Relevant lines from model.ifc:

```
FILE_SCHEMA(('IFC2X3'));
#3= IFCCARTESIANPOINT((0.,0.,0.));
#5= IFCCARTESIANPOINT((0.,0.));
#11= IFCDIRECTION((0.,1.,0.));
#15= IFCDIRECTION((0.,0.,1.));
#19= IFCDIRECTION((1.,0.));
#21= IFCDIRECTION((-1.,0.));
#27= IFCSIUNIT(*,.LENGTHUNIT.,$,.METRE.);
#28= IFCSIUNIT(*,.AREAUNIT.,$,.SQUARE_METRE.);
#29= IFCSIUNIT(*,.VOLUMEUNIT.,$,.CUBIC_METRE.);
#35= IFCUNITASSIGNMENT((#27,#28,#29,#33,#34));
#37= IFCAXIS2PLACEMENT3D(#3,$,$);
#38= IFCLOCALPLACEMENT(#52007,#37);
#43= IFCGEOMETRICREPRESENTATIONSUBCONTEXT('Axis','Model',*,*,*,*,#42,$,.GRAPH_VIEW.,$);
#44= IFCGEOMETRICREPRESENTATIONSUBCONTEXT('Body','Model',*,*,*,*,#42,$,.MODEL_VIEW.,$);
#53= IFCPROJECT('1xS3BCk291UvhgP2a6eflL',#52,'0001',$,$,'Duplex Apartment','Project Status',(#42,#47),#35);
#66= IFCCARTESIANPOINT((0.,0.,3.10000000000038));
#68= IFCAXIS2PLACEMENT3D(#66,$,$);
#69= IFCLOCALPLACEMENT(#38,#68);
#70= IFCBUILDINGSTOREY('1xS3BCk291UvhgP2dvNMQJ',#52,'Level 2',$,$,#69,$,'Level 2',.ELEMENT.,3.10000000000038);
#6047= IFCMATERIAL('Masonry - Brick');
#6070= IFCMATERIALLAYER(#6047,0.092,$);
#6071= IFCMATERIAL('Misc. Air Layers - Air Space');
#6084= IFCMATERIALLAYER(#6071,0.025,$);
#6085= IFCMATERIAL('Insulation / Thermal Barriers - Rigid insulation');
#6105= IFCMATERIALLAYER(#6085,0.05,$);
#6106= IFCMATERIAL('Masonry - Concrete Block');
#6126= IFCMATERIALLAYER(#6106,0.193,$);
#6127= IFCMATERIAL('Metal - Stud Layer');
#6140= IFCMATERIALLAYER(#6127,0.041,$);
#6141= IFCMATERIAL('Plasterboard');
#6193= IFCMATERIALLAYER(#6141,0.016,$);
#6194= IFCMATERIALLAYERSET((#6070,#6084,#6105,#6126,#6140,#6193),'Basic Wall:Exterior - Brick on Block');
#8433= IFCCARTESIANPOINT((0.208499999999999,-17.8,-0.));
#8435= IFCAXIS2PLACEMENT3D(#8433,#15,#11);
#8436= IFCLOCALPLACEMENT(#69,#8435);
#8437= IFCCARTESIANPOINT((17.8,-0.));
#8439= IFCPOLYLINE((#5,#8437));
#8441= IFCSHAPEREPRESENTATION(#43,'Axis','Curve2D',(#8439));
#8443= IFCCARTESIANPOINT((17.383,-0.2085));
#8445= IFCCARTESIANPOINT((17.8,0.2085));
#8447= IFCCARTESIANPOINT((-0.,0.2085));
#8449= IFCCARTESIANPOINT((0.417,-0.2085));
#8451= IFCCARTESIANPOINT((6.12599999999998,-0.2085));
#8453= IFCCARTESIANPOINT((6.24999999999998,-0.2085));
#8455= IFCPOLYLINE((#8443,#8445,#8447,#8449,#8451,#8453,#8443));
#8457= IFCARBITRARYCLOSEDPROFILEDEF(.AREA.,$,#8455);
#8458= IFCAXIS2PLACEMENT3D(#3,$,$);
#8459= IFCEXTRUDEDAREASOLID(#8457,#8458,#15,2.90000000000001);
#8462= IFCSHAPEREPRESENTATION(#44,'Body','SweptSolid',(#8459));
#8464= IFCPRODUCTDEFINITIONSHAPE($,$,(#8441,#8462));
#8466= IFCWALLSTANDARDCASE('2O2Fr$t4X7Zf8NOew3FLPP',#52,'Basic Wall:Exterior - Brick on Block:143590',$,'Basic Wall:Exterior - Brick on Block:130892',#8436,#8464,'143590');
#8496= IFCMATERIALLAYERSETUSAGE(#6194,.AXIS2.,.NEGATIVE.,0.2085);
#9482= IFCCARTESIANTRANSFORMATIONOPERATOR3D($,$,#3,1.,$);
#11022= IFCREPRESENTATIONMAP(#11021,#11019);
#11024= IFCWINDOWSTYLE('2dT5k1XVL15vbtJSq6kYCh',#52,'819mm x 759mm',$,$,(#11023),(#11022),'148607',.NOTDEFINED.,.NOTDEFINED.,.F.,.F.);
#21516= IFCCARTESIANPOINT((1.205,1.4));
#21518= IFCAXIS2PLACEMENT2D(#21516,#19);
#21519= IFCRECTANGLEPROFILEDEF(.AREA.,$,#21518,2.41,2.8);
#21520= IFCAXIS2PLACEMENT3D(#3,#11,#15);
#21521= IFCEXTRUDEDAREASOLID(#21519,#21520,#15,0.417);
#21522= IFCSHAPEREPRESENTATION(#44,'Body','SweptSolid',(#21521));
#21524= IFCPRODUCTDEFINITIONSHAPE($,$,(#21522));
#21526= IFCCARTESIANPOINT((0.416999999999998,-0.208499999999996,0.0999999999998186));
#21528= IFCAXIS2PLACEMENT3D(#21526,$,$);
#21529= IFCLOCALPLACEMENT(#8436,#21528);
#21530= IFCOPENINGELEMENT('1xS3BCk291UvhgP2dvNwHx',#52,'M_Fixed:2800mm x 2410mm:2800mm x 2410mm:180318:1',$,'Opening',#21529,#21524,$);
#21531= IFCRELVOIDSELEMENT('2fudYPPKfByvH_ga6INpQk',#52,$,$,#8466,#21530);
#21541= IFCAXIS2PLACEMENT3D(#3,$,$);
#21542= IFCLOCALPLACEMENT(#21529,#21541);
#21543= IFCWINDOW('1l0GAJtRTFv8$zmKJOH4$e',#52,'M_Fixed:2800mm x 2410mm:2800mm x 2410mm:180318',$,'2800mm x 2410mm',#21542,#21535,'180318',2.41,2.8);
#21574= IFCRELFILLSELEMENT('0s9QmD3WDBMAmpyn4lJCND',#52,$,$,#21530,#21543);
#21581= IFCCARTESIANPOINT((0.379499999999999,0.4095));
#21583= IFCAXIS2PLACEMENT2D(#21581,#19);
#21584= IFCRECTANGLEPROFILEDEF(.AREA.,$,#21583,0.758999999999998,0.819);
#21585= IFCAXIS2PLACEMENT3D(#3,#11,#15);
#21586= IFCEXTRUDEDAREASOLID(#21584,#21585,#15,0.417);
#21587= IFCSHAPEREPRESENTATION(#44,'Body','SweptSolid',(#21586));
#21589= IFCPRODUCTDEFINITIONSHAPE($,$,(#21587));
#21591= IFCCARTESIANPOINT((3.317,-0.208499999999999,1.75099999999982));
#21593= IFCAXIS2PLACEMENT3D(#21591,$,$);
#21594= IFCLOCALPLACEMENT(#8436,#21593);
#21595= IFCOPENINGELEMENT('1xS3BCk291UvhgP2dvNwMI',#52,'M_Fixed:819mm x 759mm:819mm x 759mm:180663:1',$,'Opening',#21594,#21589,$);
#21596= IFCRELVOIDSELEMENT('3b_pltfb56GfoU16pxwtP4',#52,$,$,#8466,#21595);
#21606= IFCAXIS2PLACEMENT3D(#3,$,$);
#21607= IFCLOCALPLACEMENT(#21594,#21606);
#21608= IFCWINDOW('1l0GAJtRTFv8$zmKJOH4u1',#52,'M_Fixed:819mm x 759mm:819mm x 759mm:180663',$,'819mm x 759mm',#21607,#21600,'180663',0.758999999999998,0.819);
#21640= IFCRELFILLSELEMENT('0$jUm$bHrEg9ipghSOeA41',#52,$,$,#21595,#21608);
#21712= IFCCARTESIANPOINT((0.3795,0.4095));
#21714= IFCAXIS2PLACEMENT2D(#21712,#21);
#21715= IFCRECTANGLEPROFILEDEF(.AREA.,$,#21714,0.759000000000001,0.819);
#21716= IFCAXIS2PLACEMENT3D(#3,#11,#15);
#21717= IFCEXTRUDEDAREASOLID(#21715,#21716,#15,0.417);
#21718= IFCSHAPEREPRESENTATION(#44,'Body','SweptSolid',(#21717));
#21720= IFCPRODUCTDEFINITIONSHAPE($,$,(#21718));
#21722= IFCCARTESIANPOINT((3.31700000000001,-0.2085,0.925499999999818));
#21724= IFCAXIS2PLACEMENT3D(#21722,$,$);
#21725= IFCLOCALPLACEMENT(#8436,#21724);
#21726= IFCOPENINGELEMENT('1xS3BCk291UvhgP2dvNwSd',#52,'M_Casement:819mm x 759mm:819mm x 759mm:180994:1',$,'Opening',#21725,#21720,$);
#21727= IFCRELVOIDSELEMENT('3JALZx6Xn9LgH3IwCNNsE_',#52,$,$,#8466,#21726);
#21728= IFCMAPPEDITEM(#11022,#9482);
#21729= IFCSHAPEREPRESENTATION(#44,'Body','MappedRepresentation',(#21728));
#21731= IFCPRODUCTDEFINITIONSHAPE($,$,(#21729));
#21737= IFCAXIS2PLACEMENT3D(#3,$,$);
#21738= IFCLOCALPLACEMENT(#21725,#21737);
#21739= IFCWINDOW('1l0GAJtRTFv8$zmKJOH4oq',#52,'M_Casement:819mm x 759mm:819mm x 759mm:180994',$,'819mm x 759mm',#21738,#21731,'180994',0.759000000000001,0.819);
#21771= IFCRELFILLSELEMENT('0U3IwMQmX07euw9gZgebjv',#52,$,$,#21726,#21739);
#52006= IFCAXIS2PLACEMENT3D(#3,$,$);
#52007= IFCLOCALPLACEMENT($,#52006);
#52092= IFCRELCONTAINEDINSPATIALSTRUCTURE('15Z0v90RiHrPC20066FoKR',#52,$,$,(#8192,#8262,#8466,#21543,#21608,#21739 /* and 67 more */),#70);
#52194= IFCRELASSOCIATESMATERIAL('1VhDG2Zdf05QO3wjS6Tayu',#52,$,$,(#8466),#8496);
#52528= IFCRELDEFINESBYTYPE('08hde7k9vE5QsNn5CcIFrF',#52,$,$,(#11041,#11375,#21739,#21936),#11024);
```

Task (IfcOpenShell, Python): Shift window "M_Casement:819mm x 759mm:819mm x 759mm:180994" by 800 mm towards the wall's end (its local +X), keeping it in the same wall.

```python
import ifcopenshell
import ifcopenshell.api.geometry
import ifcopenshell.util.placement

model = ifcopenshell.open("model.ifc")

window = model.by_guid("1l0GAJtRTFv8$zmKJOH4oq")
opening = window.FillsVoids[0].RelatingOpeningElement
wall = opening.VoidsElements[0].RelatingBuildingElement

wall_matrix = ifcopenshell.util.placement.get_local_placement(wall.ObjectPlacement)
shift = wall_matrix[:3, 0] * 0.8
before = ifcopenshell.util.placement.get_local_placement(window.ObjectPlacement)[:3, 3].copy()

# The window is placed relative to its opening, so it follows when the opening moves.
matrix = ifcopenshell.util.placement.get_local_placement(opening.ObjectPlacement)
matrix[:3, 3] += shift
ifcopenshell.api.geometry.edit_object_placement(
    model, product=opening, matrix=matrix, is_si=False, should_transform_children=True
)

after = ifcopenshell.util.placement.get_local_placement(window.ObjectPlacement)[:3, 3]
print("window moved by", (after - before).round(3) + 0.0)

model.write("model_updated.ifc")
```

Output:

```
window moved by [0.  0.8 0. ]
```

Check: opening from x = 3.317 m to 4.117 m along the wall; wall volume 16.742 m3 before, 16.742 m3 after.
